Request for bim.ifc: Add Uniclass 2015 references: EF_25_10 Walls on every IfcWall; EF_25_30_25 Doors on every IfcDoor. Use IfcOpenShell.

First a look at what the model holds.

```python
import ifcopenshell

model = ifcopenshell.open("bim.ifc")
print(model.schema)
print("classifications:", [c.Name for c in model.by_type("IfcClassification")])
for ifc_class in ("IfcDoor", "IfcRoof", "IfcStair", "IfcWall", "IfcWindow"):
    print(ifc_class, len(model.by_type(ifc_class)))
```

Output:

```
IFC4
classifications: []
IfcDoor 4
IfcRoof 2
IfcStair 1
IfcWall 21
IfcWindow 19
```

```python
import ifcopenshell
import ifcopenshell.api.classification

model = ifcopenshell.open("bim.ifc")

system = ifcopenshell.api.classification.add_classification(model, classification="Uniclass 2015")

codes = {
    "IfcWall": ("EF_25_10", "Walls"),
    "IfcDoor": ("EF_25_30_25", "Doors"),
}
for ifc_class, (code, name) in codes.items():
    products = model.by_type(ifc_class)
    ifcopenshell.api.classification.add_reference(
        model, products=products, classification=system, identification=code, name=name
    )
    print(code, len(products))

model.write("bim_edited.ifc")
```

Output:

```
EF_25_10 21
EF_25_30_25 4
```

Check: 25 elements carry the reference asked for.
